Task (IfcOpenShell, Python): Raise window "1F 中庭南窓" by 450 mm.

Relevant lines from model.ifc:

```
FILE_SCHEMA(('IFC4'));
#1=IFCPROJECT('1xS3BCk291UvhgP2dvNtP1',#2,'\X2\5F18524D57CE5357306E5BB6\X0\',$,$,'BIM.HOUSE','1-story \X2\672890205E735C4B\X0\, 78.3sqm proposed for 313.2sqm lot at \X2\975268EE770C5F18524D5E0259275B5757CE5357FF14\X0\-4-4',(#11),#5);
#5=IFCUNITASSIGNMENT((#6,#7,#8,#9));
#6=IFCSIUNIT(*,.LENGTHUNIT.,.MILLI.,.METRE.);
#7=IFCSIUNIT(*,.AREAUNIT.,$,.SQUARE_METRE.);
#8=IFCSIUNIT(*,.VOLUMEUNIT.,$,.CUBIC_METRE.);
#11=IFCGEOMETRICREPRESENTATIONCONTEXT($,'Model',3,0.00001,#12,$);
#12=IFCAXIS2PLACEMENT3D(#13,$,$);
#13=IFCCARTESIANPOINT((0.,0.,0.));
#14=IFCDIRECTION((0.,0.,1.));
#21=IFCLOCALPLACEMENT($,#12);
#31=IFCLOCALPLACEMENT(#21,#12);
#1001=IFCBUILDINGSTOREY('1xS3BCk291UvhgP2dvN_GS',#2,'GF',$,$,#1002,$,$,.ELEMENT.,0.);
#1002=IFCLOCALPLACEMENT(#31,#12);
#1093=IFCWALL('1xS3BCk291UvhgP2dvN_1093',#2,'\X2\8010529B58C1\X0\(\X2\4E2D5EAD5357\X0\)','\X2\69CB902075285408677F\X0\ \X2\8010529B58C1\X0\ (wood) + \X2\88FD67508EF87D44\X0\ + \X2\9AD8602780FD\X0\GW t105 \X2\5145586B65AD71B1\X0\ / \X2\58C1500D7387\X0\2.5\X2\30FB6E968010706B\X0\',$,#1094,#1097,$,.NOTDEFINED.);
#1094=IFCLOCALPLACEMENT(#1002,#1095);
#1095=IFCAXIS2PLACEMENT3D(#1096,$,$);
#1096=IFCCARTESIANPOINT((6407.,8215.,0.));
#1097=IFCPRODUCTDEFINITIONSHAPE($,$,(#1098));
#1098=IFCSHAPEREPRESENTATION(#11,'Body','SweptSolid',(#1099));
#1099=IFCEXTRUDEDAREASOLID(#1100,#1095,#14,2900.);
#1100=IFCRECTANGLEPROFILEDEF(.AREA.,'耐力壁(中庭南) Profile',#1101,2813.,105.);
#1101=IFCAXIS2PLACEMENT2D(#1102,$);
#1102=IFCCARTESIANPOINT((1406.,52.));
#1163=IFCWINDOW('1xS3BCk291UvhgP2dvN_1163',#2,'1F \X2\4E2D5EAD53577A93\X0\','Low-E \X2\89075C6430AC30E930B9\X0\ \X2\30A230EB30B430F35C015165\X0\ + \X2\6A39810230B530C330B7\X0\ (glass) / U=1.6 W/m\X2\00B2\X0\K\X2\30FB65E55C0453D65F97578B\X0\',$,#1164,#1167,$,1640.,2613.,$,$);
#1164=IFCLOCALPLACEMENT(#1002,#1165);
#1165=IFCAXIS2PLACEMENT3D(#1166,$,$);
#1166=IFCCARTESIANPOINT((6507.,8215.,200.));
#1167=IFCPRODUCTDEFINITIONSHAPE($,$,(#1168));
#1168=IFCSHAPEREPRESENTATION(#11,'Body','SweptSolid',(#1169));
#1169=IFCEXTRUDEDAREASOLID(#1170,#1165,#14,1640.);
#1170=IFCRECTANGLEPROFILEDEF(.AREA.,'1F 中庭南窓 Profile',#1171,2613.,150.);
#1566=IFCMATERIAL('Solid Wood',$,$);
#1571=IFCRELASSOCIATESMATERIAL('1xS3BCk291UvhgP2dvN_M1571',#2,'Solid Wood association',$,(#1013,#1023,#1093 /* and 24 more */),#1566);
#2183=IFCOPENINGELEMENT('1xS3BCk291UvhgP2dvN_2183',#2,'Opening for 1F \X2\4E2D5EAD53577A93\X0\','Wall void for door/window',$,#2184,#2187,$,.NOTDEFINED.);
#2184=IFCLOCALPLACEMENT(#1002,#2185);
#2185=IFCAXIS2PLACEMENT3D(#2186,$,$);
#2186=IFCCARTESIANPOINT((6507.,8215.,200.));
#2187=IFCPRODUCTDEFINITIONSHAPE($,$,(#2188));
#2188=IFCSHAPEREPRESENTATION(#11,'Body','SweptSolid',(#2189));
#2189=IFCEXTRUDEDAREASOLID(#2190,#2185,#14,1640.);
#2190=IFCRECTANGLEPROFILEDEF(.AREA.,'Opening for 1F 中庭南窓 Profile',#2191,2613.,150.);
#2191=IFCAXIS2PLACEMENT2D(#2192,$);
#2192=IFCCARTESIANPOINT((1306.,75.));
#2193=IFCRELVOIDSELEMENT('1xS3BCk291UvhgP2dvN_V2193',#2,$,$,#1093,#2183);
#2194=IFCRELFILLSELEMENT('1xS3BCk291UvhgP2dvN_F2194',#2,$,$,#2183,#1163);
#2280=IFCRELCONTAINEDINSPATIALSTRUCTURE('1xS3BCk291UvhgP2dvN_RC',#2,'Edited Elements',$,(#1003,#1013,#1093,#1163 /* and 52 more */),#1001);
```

```python
import numpy as np
import ifcopenshell
import ifcopenshell.api.geometry
import ifcopenshell.util.placement
import ifcopenshell.util.unit

model = ifcopenshell.open("model.ifc")
unit_scale = ifcopenshell.util.unit.calculate_unit_scale(model)

window = model.by_id(1163)
opening = window.FillsVoids[0].RelatingOpeningElement
dz = 0.45 / unit_scale

shift = np.array([0.0, 0.0, dz])
# The window is not placed relative to its opening, so move both.
for product in (opening, window):
    matrix = ifcopenshell.util.placement.get_local_placement(product.ObjectPlacement)
    matrix[:3, 3] += shift
    ifcopenshell.api.geometry.edit_object_placement(model, product=product, matrix=matrix, is_si=False)

print(f"moved by {dz * unit_scale:+.3f} m")

model.write("model_edited.ifc")
```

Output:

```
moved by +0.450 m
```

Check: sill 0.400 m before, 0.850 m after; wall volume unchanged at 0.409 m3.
